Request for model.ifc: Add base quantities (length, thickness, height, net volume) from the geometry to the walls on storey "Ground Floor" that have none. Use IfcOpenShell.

First a look at what the model holds.

```python
import ifcopenshell
import ifcopenshell.util.element
import ifcopenshell.util.unit

model = ifcopenshell.open("model.ifc")
print(model.schema)
for unit_type in ("LENGTHUNIT", "AREAUNIT", "VOLUMEUNIT"):
    print(unit_type, ifcopenshell.util.unit.calculate_unit_scale(model, unit_type))
storey = next(s for s in model.by_type("IfcBuildingStorey") if s.Name == "Ground Floor")
walls = [e for e in ifcopenshell.util.element.get_decomposition(storey) if e.is_a("IfcWall")]
for e in sorted(walls, key=lambda e: e.id()):
    print(e.id(), e.is_a(), e.Name, list(ifcopenshell.util.element.get_psets(e, qtos_only=True)), sep=" | ")
```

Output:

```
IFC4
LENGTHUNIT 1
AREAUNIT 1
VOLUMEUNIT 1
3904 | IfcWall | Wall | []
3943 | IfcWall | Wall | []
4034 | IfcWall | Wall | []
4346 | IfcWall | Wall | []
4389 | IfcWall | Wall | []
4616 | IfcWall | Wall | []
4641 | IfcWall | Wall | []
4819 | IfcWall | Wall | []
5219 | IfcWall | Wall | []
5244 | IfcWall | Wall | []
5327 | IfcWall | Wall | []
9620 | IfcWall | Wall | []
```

```python
import ifcopenshell
import ifcopenshell.api.pset
import ifcopenshell.geom
import ifcopenshell.util.element
import ifcopenshell.util.shape
import ifcopenshell.util.unit

model = ifcopenshell.open("model.ifc")
unit_scale = ifcopenshell.util.unit.calculate_unit_scale(model)
volume_scale = ifcopenshell.util.unit.calculate_unit_scale(model, "VOLUMEUNIT")
settings = ifcopenshell.geom.settings()

storey = next(s for s in model.by_type("IfcBuildingStorey") if s.Name == "Ground Floor")
walls = [e for e in ifcopenshell.util.element.get_decomposition(storey) if e.is_a("IfcWall")]

for e in sorted(walls, key=lambda e: e.id()):
    if ifcopenshell.util.element.get_psets(e, qtos_only=True, should_inherit=False):
        continue
    # Geometry comes back in metres, in the element's own axes.
    shape = ifcopenshell.geom.create_shape(settings, e)
    values = {
        "Length": ifcopenshell.util.shape.get_x(shape.geometry) / unit_scale,
        "Width": ifcopenshell.util.shape.get_y(shape.geometry) / unit_scale,
        "Height": ifcopenshell.util.shape.get_z(shape.geometry) / unit_scale,
        "NetVolume": ifcopenshell.util.shape.get_volume(shape.geometry) / volume_scale,
    }
    qto = ifcopenshell.api.pset.add_qto(model, product=e, name="Qto_WallBaseQuantities")
    ifcopenshell.api.pset.edit_qto(model, qto=qto, properties=values)
    print(e.id(), {k: round(v, 3) for k, v in values.items()})

model.write("model_rev.ifc")
```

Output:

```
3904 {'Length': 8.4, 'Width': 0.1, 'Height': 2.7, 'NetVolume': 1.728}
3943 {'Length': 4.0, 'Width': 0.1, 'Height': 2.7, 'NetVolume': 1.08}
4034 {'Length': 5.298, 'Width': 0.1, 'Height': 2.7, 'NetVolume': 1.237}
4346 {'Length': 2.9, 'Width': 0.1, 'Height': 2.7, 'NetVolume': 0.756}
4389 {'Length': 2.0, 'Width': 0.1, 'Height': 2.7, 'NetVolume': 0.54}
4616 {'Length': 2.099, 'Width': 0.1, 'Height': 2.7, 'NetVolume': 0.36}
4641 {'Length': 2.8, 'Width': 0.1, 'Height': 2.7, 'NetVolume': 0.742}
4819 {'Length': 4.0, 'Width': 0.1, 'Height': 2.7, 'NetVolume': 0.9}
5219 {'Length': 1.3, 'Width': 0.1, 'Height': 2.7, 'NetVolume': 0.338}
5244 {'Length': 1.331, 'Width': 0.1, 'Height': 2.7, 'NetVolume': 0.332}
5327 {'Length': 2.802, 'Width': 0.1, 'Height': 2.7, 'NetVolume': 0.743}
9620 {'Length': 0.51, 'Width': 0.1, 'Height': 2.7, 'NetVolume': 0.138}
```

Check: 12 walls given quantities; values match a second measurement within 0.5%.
